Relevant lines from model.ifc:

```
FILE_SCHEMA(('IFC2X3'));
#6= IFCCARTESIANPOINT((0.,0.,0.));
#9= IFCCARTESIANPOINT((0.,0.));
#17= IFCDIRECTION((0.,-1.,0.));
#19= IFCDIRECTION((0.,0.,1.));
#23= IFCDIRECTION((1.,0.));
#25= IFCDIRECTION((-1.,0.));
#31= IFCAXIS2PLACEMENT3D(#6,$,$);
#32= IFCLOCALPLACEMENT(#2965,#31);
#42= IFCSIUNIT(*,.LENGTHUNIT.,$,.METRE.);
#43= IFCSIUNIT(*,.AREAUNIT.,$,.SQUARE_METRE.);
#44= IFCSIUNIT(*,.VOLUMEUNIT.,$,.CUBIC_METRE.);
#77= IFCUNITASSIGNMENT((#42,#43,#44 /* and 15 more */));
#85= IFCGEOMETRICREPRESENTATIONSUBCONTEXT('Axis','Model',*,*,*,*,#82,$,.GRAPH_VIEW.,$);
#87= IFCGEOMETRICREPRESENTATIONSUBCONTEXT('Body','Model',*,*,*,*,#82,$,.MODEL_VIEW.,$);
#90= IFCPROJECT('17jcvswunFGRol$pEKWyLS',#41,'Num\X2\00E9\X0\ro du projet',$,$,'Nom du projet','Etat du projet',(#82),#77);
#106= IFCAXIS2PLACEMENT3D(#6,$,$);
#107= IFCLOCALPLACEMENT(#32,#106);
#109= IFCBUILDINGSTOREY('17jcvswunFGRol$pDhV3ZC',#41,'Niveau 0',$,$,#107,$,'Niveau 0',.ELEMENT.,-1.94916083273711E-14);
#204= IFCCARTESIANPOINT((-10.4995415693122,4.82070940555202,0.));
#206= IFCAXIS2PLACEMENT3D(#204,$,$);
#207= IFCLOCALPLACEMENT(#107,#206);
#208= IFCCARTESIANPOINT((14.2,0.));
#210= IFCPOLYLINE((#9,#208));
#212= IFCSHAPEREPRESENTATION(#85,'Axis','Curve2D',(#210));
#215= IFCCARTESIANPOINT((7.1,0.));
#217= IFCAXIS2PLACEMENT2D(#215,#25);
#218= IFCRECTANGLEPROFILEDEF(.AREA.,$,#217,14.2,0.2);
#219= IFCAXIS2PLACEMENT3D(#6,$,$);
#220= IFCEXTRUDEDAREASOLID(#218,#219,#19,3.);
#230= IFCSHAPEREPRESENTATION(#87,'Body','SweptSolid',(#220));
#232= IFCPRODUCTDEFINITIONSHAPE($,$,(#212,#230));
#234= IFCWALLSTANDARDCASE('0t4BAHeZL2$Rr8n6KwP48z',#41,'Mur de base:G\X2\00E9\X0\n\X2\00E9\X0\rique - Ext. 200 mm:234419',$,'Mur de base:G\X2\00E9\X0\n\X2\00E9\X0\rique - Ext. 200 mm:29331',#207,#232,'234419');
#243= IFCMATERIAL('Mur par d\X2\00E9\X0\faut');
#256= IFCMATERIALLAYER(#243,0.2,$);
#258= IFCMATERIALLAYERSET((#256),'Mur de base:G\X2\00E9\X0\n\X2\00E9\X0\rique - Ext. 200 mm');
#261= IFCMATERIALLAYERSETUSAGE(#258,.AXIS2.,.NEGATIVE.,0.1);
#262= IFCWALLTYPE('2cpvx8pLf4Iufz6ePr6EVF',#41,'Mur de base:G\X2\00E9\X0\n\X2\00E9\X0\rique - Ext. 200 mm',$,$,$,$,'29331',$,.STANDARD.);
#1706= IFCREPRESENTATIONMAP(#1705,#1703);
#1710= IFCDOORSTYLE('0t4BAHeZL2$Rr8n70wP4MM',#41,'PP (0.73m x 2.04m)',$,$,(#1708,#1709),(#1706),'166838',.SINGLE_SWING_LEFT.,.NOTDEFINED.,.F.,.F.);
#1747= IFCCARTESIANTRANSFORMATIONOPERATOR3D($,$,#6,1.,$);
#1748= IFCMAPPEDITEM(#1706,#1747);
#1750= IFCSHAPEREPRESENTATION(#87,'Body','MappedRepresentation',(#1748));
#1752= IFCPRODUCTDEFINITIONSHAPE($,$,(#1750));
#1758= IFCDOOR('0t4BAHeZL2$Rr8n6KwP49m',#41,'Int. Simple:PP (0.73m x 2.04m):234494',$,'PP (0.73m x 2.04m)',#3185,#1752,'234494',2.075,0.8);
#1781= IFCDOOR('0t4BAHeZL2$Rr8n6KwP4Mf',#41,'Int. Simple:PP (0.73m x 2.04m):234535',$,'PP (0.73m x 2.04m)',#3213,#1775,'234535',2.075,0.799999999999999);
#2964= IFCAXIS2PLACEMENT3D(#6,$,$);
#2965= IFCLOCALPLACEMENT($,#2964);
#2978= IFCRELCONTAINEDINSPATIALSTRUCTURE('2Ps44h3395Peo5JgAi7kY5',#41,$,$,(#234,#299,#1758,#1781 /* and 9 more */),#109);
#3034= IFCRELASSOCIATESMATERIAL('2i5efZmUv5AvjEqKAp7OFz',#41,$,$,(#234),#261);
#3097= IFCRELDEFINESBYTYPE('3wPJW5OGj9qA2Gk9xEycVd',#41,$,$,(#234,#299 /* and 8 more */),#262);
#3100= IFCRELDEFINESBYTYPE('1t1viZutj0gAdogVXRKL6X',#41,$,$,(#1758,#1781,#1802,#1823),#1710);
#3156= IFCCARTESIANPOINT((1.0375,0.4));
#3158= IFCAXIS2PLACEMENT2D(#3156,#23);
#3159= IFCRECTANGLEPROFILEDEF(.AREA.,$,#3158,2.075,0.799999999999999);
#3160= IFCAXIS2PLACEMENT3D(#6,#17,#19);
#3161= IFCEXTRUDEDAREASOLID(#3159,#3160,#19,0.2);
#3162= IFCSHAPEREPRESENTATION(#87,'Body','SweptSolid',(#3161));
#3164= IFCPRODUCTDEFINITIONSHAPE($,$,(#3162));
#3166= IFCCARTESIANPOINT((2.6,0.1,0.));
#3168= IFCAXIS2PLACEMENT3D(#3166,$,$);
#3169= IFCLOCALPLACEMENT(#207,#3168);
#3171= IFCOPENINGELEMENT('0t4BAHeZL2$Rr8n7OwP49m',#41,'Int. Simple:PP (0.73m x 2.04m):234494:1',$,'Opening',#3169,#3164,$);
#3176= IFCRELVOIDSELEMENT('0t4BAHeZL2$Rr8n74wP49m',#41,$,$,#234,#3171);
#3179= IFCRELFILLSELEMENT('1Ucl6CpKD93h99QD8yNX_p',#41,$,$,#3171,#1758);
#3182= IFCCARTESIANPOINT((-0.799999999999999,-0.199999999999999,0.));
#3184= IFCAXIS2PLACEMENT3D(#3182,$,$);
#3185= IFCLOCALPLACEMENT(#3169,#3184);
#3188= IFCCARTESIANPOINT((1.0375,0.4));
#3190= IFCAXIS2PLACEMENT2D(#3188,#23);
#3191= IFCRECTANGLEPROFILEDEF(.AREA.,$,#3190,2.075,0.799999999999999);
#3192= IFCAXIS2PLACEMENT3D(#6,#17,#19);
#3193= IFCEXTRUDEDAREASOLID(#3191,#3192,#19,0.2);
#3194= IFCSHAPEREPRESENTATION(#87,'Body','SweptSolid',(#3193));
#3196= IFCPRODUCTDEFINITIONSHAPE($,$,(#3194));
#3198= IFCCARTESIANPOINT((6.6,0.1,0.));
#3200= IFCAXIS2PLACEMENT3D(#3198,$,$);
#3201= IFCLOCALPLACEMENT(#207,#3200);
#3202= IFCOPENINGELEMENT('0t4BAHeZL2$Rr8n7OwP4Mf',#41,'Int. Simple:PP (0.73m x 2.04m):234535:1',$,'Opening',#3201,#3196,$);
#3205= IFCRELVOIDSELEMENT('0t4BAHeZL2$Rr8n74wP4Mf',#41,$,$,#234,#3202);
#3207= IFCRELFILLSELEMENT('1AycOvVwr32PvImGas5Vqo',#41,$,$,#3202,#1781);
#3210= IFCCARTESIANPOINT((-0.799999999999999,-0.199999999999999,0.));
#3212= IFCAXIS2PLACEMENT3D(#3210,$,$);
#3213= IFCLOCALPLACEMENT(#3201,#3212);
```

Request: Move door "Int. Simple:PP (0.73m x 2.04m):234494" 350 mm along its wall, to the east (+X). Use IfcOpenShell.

```python
import ifcopenshell
import ifcopenshell.api.geometry
import ifcopenshell.util.placement
import ifcopenshell.util.unit

model = ifcopenshell.open("model.ifc")
unit_scale = ifcopenshell.util.unit.calculate_unit_scale(model)

door = model.by_guid("0t4BAHeZL2$Rr8n6KwP49m")
opening = door.FillsVoids[0].RelatingOpeningElement
wall = opening.VoidsElements[0].RelatingBuildingElement

wall_matrix = ifcopenshell.util.placement.get_local_placement(wall.ObjectPlacement)
shift = wall_matrix[:3, 0] * 0.35 / unit_scale
before = ifcopenshell.util.placement.get_local_placement(door.ObjectPlacement)[:3, 3].copy()

# The door is placed relative to its opening, so it follows when the opening moves.
matrix = ifcopenshell.util.placement.get_local_placement(opening.ObjectPlacement)
matrix[:3, 3] += shift
ifcopenshell.api.geometry.edit_object_placement(
    model, product=opening, matrix=matrix, is_si=False, should_transform_children=True
)

after = ifcopenshell.util.placement.get_local_placement(door.ObjectPlacement)[:3, 3]
print("door moved by", (after - before).round(3) + 0.0)

model.write("model_updated.ifc")
```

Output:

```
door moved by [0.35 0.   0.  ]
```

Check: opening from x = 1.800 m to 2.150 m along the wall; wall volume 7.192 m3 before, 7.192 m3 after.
